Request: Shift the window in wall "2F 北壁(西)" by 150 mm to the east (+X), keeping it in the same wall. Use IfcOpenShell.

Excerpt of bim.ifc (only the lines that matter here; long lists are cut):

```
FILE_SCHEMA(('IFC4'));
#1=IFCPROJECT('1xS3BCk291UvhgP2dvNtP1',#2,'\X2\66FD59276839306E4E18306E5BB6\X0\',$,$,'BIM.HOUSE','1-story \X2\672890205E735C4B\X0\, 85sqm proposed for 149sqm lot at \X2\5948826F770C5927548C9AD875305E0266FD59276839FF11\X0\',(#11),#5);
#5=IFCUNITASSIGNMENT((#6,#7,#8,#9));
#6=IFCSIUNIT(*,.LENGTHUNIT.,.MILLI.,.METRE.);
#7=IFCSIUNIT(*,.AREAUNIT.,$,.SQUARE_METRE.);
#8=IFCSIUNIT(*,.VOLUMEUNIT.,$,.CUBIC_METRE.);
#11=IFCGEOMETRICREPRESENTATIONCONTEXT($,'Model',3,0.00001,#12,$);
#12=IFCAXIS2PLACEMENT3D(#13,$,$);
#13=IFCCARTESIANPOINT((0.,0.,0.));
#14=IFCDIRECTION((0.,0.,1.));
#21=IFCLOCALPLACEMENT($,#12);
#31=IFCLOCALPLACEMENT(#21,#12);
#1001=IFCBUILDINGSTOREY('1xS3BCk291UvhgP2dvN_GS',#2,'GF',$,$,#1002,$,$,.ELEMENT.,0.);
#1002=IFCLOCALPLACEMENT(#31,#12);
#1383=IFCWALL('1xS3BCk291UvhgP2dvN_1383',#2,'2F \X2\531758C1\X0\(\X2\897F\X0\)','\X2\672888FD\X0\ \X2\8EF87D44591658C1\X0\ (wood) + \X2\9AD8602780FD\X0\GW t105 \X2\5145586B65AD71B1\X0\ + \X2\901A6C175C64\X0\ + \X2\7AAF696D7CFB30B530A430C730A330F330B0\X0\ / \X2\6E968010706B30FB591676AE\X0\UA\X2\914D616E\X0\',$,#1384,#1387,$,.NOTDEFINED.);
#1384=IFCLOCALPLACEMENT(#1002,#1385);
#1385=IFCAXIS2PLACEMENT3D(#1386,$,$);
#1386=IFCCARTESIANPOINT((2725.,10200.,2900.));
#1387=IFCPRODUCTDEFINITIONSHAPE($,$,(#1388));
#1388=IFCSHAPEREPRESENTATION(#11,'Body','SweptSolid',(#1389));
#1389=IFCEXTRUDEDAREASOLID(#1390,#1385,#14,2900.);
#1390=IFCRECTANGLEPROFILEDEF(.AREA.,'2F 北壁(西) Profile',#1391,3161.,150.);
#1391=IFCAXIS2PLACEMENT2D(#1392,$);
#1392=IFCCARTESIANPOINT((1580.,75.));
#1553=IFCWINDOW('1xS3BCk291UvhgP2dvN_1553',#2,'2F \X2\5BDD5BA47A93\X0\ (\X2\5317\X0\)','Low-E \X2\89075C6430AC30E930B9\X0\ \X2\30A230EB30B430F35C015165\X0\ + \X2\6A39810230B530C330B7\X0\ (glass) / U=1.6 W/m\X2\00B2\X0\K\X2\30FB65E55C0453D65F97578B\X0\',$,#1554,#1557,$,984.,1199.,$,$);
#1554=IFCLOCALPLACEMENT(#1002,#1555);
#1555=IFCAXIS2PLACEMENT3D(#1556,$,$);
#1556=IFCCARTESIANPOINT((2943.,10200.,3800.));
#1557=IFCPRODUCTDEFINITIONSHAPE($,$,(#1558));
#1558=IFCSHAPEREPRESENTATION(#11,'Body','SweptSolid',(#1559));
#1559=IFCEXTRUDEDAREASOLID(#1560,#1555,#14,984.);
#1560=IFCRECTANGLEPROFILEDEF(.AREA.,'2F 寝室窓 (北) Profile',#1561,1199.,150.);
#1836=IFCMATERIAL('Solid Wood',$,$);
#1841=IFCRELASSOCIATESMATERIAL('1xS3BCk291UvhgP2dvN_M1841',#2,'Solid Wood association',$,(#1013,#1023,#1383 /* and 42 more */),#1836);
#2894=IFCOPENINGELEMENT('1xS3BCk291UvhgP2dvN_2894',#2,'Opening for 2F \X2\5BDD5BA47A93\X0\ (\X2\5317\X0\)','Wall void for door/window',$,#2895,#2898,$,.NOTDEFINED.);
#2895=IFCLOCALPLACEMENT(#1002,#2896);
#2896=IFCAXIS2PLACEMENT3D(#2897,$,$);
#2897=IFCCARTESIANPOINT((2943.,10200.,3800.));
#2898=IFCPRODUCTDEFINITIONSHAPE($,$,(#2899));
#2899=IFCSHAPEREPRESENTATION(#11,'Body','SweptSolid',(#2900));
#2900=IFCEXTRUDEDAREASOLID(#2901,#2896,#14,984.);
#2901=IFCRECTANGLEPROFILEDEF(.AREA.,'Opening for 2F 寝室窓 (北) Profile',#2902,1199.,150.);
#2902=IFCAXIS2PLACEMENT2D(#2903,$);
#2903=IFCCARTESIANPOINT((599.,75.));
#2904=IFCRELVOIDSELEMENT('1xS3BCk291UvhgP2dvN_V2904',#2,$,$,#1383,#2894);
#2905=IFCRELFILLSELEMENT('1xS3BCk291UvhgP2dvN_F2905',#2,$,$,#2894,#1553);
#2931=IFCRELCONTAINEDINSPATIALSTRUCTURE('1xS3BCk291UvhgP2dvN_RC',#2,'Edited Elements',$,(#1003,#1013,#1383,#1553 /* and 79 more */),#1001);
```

```python
import ifcopenshell
import ifcopenshell.api.geometry
import ifcopenshell.util.placement
import ifcopenshell.util.unit

model = ifcopenshell.open("bim.ifc")
unit_scale = ifcopenshell.util.unit.calculate_unit_scale(model)

window = model.by_id(1553)
opening = window.FillsVoids[0].RelatingOpeningElement
wall = opening.VoidsElements[0].RelatingBuildingElement

wall_matrix = ifcopenshell.util.placement.get_local_placement(wall.ObjectPlacement)
shift = wall_matrix[:3, 0] * 0.15 / unit_scale
before = ifcopenshell.util.placement.get_local_placement(window.ObjectPlacement)[:3, 3].copy()

# The window is not placed relative to its opening, so move both.
for product in (opening, window):
    matrix = ifcopenshell.util.placement.get_local_placement(product.ObjectPlacement)
    matrix[:3, 3] += shift
    ifcopenshell.api.geometry.edit_object_placement(model, product=product, matrix=matrix, is_si=False)

after = ifcopenshell.util.placement.get_local_placement(window.ObjectPlacement)[:3, 3]
print("window moved by", (after - before).round(3) + 0.0)

model.write("bim-out.ifc")
```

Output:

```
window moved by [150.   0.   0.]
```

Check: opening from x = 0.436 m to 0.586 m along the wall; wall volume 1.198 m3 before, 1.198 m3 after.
